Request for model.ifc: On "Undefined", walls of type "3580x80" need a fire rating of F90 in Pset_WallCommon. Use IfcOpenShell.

First a look at what the model holds.

```python
import ifcopenshell
import ifcopenshell.util.element

model = ifcopenshell.open("model.ifc")
print(model.schema)
storey = next(s for s in model.by_type("IfcBuildingStorey") if s.Name == "Undefined")
walls = [e for e in ifcopenshell.util.element.get_decomposition(storey) if e.is_a("IfcWall")]
seen = {}
for e in walls:
    element_type = ifcopenshell.util.element.get_type(e)
    key = (element_type.Name if element_type != e and element_type else None, ifcopenshell.util.element.get_pset(e, "Pset_WallCommon", "FireRating"))
    seen[key] = seen.get(key, 0) + 1
for (name, value), count in sorted(seen.items(), key=str):
    print(count, "x", name, "|", value)
```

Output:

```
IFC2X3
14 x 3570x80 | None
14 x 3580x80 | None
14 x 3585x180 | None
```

```python
import ifcopenshell
import ifcopenshell.api.pset
import ifcopenshell.util.element

model = ifcopenshell.open("model.ifc")

storey = next(s for s in model.by_type("IfcBuildingStorey") if s.Name == "Undefined")
walls = [e for e in ifcopenshell.util.element.get_decomposition(storey) if e.is_a("IfcWall")]

count = 0
for e in walls:
    element_type = ifcopenshell.util.element.get_type(e)
    if element_type in (None, e) or element_type.Name != "3580x80":
        continue
    found = ifcopenshell.util.element.get_pset(e, "Pset_WallCommon", should_inherit=False)
    if found:
        pset = model.by_id(found["id"])
        if len(ifcopenshell.util.element.get_elements_by_pset(pset)) > 1:
            pset = ifcopenshell.api.pset.unshare_pset(model, products=[e], pset=pset)[0]
    else:
        pset = ifcopenshell.api.pset.add_pset(model, product=e, name="Pset_WallCommon")
    ifcopenshell.api.pset.edit_pset(model, pset=pset, properties={"FireRating": "F90"})
    count += 1

print(count, "walls updated")

model.write("model-out.ifc")
```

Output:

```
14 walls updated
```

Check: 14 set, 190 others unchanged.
